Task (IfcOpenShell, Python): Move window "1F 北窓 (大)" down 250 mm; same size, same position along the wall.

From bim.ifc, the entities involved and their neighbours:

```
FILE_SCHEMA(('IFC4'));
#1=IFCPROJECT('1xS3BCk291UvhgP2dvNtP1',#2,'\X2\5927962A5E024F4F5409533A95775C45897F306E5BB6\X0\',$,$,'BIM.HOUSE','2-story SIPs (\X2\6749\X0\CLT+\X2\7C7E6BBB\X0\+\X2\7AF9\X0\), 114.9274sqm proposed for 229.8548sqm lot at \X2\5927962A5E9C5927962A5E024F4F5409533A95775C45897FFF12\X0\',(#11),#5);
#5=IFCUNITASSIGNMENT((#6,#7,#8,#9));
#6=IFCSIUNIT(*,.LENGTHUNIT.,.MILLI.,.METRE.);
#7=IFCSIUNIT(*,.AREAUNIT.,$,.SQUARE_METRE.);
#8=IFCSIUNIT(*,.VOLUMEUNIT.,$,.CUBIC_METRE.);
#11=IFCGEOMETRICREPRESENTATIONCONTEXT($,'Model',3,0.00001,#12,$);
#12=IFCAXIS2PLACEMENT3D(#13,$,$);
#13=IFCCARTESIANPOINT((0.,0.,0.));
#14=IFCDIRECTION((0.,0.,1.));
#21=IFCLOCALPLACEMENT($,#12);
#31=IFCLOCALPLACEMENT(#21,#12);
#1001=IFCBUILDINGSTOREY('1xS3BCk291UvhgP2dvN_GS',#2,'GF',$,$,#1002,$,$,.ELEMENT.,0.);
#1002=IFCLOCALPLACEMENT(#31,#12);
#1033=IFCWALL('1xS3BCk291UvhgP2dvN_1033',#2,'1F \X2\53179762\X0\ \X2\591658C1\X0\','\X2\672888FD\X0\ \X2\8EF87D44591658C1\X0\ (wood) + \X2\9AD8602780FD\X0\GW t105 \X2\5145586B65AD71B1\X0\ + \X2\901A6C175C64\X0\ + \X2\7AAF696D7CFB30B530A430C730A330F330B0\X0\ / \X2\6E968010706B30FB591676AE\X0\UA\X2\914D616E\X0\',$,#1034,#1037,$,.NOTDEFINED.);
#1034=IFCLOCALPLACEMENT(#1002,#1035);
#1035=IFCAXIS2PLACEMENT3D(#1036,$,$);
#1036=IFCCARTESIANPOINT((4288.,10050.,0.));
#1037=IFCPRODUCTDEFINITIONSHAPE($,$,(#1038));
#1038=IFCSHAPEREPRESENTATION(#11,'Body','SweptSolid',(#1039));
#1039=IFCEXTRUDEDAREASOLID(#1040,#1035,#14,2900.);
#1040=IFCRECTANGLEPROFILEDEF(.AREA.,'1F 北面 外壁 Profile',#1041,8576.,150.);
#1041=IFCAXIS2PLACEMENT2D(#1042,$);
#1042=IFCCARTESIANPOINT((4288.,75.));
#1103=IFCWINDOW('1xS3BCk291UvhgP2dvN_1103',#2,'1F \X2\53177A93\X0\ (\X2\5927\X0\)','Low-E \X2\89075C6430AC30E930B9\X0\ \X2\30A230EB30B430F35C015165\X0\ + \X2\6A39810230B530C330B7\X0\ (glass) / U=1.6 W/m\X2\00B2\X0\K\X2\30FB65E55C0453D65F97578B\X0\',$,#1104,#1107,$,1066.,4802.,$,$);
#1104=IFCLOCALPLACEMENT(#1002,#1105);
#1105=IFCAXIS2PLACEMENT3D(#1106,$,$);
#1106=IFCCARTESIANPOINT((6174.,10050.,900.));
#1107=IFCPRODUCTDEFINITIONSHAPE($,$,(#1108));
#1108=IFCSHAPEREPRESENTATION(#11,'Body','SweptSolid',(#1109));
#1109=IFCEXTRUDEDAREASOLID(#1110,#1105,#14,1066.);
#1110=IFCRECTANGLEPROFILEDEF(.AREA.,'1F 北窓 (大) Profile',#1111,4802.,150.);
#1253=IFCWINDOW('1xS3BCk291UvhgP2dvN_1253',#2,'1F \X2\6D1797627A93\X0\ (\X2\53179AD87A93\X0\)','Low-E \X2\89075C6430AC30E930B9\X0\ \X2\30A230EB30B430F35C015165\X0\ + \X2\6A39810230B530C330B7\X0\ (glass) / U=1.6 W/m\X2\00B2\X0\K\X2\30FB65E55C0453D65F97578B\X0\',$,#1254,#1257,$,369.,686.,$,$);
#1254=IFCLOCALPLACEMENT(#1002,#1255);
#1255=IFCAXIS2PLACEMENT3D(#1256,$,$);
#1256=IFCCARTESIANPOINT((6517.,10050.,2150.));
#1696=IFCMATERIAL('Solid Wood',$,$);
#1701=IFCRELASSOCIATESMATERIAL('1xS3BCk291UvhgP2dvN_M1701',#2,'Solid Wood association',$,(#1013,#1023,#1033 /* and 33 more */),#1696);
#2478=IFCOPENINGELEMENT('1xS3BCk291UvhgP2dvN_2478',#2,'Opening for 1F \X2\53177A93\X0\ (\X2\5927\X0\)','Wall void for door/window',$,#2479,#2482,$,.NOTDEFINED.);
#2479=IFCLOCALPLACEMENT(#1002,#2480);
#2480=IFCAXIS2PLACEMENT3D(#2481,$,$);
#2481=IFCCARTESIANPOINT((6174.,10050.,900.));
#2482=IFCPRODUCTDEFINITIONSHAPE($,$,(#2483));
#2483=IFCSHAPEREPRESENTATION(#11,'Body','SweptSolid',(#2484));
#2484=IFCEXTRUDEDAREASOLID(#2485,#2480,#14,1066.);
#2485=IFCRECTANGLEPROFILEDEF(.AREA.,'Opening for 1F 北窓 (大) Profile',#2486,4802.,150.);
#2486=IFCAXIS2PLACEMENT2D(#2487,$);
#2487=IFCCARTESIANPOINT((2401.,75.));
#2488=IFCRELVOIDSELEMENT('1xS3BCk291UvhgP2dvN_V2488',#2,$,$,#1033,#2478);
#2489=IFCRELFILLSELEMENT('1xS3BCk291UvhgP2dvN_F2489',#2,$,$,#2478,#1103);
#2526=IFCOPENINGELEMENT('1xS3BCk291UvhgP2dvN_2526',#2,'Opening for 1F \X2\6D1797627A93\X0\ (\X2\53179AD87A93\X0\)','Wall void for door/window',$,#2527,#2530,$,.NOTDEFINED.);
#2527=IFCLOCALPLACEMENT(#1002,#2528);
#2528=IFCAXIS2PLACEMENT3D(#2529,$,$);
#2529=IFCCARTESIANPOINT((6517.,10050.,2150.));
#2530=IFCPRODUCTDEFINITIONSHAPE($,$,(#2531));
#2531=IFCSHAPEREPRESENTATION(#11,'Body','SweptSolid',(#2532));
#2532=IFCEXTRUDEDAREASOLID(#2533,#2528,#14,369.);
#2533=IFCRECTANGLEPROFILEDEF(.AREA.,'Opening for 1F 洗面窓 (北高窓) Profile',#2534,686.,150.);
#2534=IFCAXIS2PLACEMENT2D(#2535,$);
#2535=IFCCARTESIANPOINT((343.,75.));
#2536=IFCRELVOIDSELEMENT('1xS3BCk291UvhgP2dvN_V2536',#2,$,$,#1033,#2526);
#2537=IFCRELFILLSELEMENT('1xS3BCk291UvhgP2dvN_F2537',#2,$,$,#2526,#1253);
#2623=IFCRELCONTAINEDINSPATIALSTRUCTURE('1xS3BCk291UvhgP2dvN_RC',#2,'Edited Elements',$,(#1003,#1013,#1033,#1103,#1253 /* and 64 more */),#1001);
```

```python
import numpy as np
import ifcopenshell
import ifcopenshell.api.geometry
import ifcopenshell.util.placement
import ifcopenshell.util.unit

model = ifcopenshell.open("bim.ifc")
unit_scale = ifcopenshell.util.unit.calculate_unit_scale(model)

window = model.by_guid("1xS3BCk291UvhgP2dvN_1103")
opening = window.FillsVoids[0].RelatingOpeningElement
dz = -0.25 / unit_scale

shift = np.array([0.0, 0.0, dz])
# The window is not placed relative to its opening, so move both.
for product in (opening, window):
    matrix = ifcopenshell.util.placement.get_local_placement(product.ObjectPlacement)
    matrix[:3, 3] += shift
    ifcopenshell.api.geometry.edit_object_placement(model, product=product, matrix=matrix, is_si=False)

print(f"moved by {dz * unit_scale:+.3f} m")

model.write("bim-out.ifc")
```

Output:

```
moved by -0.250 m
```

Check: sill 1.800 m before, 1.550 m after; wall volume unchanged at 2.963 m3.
